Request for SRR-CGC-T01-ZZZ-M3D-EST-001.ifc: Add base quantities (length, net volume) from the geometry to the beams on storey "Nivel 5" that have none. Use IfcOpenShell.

First a look at what the model holds.

```python
import ifcopenshell
import ifcopenshell.util.element
import ifcopenshell.util.unit

model = ifcopenshell.open("SRR-CGC-T01-ZZZ-M3D-EST-001.ifc")
print(model.schema)
for unit_type in ("LENGTHUNIT", "AREAUNIT", "VOLUMEUNIT"):
    print(unit_type, ifcopenshell.util.unit.calculate_unit_scale(model, unit_type))
storey = next(s for s in model.by_type("IfcBuildingStorey") if s.Name == "Nivel 5")
beams = [e for e in ifcopenshell.util.element.get_decomposition(storey) if e.is_a("IfcBeam")]
for e in sorted(beams, key=lambda e: e.id()):
    print(e.id(), e.is_a(), e.Name, list(ifcopenshell.util.element.get_psets(e, qtos_only=True)), sep=" | ")
```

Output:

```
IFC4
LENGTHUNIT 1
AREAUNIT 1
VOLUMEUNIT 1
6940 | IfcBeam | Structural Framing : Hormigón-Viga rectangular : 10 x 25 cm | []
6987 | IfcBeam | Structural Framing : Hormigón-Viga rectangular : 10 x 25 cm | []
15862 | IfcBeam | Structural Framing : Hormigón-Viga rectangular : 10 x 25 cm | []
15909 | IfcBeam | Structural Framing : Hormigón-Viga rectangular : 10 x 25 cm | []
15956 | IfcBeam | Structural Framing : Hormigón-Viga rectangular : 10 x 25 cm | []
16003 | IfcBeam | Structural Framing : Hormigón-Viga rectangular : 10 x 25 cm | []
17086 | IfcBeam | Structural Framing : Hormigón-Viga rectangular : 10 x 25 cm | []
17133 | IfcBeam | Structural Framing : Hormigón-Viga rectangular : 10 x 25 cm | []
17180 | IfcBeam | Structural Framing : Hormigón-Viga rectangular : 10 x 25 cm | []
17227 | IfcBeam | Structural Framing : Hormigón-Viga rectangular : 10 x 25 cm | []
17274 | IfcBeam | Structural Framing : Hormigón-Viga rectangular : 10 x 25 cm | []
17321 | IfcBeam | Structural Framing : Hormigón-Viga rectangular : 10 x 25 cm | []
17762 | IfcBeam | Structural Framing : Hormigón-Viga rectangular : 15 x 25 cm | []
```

```python
import ifcopenshell
import ifcopenshell.api.pset
import ifcopenshell.geom
import ifcopenshell.util.element
import ifcopenshell.util.shape
import ifcopenshell.util.unit

model = ifcopenshell.open("SRR-CGC-T01-ZZZ-M3D-EST-001.ifc")
unit_scale = ifcopenshell.util.unit.calculate_unit_scale(model)
volume_scale = ifcopenshell.util.unit.calculate_unit_scale(model, "VOLUMEUNIT")
settings = ifcopenshell.geom.settings()

storey = next(s for s in model.by_type("IfcBuildingStorey") if s.Name == "Nivel 5")
beams = [e for e in ifcopenshell.util.element.get_decomposition(storey) if e.is_a("IfcBeam")]

for e in sorted(beams, key=lambda e: e.id()):
    if ifcopenshell.util.element.get_psets(e, qtos_only=True, should_inherit=False):
        continue
    # Geometry comes back in metres, in the element's own axes.
    shape = ifcopenshell.geom.create_shape(settings, e)
    values = {
        "Length": ifcopenshell.util.shape.get_max_xyz(shape.geometry) / unit_scale,
        "NetVolume": ifcopenshell.util.shape.get_volume(shape.geometry) / volume_scale,
    }
    qto = ifcopenshell.api.pset.add_qto(model, product=e, name="Qto_BeamBaseQuantities")
    ifcopenshell.api.pset.edit_qto(model, qto=qto, properties=values)
    print(e.id(), {k: round(v, 3) for k, v in values.items()})

model.write("SRR-CGC-T01-ZZZ-M3D-EST-001_edited.ifc")
```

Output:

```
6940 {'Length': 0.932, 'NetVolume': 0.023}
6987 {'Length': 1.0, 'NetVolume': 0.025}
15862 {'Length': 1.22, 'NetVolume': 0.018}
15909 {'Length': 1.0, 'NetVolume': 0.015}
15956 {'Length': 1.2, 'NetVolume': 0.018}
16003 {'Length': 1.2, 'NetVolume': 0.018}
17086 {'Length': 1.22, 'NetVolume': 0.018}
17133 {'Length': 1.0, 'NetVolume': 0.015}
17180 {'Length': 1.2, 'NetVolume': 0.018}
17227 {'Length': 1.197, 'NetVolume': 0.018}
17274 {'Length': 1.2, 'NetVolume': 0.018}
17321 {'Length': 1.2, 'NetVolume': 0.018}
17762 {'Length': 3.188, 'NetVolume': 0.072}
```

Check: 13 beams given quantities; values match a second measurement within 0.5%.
